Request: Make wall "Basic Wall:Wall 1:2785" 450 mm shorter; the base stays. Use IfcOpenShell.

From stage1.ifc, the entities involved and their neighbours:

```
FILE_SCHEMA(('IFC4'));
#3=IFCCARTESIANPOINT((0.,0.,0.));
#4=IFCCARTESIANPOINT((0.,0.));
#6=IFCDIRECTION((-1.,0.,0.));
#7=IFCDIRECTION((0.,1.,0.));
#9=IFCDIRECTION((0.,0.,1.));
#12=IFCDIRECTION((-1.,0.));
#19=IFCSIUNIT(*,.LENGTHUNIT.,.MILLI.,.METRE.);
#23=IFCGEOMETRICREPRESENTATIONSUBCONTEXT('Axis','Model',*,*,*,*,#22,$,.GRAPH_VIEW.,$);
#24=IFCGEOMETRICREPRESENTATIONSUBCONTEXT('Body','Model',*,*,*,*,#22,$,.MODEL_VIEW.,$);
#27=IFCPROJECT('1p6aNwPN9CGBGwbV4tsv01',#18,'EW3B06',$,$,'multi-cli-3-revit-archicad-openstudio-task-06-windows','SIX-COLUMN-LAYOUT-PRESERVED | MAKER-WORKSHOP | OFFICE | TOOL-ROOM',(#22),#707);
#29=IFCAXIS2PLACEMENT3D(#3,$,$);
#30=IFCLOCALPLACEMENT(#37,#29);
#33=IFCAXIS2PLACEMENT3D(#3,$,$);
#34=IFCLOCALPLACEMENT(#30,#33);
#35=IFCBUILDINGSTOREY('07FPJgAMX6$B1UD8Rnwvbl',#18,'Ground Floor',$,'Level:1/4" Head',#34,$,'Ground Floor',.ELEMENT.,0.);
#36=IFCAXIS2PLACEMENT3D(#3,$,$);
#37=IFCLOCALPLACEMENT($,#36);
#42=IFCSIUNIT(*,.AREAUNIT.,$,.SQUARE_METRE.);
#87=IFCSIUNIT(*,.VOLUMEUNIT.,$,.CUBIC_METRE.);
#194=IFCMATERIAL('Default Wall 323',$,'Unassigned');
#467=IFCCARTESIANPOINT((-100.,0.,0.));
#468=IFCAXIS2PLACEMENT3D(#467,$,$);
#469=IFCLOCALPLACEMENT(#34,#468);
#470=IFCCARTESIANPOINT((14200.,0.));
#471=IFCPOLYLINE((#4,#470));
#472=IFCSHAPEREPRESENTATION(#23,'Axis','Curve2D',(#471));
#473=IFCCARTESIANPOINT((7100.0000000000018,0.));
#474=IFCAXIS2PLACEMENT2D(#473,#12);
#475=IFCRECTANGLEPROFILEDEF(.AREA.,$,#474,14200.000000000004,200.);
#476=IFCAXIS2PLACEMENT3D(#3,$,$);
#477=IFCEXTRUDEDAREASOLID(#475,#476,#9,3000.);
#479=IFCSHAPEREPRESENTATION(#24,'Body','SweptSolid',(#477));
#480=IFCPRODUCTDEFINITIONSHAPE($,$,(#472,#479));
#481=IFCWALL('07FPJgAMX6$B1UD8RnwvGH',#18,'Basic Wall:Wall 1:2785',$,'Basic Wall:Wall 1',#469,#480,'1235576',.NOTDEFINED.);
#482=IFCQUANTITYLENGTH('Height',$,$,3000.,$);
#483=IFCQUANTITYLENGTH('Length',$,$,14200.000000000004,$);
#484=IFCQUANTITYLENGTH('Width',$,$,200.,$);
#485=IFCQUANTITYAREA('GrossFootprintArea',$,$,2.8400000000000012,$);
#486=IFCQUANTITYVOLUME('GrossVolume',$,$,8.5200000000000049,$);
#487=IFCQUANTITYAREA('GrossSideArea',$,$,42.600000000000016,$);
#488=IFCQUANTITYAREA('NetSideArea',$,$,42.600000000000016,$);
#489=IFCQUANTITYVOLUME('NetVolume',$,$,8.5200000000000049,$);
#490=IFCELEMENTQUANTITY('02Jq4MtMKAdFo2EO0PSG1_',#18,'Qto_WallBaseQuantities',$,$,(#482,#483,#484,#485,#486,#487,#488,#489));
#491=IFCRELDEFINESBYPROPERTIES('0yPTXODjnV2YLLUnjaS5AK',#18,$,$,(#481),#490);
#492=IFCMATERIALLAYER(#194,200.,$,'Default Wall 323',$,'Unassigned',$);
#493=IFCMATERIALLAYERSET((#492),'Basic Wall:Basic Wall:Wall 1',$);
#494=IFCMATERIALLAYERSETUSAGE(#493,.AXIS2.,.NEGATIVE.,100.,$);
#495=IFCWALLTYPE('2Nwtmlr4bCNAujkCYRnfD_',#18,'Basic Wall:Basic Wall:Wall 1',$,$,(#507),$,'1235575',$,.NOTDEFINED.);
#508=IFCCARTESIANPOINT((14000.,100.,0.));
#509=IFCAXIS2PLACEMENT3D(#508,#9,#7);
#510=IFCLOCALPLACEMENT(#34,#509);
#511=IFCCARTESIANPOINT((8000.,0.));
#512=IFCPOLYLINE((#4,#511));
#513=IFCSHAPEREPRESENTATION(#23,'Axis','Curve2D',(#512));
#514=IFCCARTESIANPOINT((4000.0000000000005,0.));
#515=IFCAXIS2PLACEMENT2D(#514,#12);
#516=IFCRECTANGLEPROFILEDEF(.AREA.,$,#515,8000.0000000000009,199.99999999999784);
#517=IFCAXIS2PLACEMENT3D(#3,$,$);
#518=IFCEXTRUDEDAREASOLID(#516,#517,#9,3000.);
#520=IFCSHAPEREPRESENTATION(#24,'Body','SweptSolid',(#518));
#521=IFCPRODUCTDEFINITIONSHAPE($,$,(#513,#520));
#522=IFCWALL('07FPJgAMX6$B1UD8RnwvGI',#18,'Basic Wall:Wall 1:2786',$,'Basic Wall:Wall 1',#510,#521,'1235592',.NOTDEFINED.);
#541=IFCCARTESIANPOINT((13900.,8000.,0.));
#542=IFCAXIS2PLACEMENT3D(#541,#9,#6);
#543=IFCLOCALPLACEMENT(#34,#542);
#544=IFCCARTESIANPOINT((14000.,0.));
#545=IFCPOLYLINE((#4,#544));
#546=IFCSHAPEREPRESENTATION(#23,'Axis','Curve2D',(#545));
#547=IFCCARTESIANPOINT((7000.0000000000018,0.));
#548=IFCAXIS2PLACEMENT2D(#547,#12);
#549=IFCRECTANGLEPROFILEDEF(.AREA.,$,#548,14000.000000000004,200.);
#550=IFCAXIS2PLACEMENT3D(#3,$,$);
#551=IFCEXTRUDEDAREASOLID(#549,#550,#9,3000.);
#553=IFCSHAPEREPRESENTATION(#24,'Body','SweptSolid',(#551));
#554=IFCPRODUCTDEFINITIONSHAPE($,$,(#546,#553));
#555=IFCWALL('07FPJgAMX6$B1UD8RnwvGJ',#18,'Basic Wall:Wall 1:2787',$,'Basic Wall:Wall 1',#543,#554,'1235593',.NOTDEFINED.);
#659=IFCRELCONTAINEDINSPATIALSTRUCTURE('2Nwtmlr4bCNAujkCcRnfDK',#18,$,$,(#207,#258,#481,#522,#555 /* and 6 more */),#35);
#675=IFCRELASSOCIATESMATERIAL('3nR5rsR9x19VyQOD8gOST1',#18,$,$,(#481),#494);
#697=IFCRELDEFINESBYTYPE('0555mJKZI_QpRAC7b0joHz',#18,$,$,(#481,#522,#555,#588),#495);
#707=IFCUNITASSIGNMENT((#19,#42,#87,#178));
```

```python
import ifcopenshell
import ifcopenshell.api.pset
import ifcopenshell.geom
import ifcopenshell.util.element
import ifcopenshell.util.representation
import ifcopenshell.util.shape
import ifcopenshell.util.unit

model = ifcopenshell.open("stage1.ifc")
unit_scale = ifcopenshell.util.unit.calculate_unit_scale(model)
area_scale = ifcopenshell.util.unit.calculate_unit_scale(model, "AREAUNIT")
volume_scale = ifcopenshell.util.unit.calculate_unit_scale(model, "VOLUMEUNIT")
settings = ifcopenshell.geom.settings()


def volume(element):
    """Net volume in cubic metres, openings subtracted."""
    shape = ifcopenshell.geom.create_shape(settings, element)
    return ifcopenshell.util.shape.get_volume(shape.geometry)


wall = model.by_guid("07FPJgAMX6$B1UD8RnwvGH")
before = volume(wall)

body = ifcopenshell.util.representation.get_representation(wall, "Model", "Body")
solid = body.Items[0]
old_height = solid.Depth
solid.Depth -= 450.0
after = volume(wall)
thickness = 0.2  # wall thickness in metres

# Update the stored height, areas and volumes.
qto = model.by_id(ifcopenshell.util.element.get_pset(wall, "Qto_WallBaseQuantities", should_inherit=False)["id"])
ifcopenshell.api.pset.edit_qto(model, qto=qto, properties={
    "Height": solid.Depth,
    "GrossVolume": ifcopenshell.util.element.get_pset(wall, "Qto_WallBaseQuantities", "GrossVolume") * solid.Depth / old_height,
    "GrossSideArea": ifcopenshell.util.element.get_pset(wall, "Qto_WallBaseQuantities", "GrossSideArea") * solid.Depth / old_height,
    "NetSideArea": after / thickness / area_scale,
    "NetVolume": after / volume_scale,
})

print(f"height {old_height:g} -> {solid.Depth:g}, volume {before:.3f} -> {after:.3f} m3")

model.write("stage1_v2.ifc")
```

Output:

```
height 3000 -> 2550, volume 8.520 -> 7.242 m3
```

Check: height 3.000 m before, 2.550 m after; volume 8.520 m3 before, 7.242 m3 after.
